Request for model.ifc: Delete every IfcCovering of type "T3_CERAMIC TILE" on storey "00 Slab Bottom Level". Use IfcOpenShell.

First a look at what the model holds.

```python
import ifcopenshell
import ifcopenshell.util.element

model = ifcopenshell.open("model.ifc")
print(model.schema)
storey = next(s for s in model.by_type("IfcBuildingStorey") if s.Name == "00 Slab Bottom Level")
coverings = [e for e in ifcopenshell.util.element.get_decomposition(storey) if e.is_a("IfcCovering")]
seen = {}
for e in coverings:
    element_type = ifcopenshell.util.element.get_type(e)
    name = element_type.Name if element_type not in (None, e) else None
    seen[name] = seen.get(name, 0) + 1
for name, count in sorted(seen.items(), key=str):
    print(count, "x", name)
```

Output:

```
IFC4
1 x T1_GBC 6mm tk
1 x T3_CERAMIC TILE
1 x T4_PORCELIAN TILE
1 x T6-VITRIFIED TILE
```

```python
import ifcopenshell
import ifcopenshell.api.root
import ifcopenshell.util.element

model = ifcopenshell.open("model.ifc")

storey = next(s for s in model.by_type("IfcBuildingStorey") if s.Name == "00 Slab Bottom Level")
coverings = [e for e in ifcopenshell.util.element.get_decomposition(storey) if e.is_a("IfcCovering")]
targets = [e for e in coverings if (t := ifcopenshell.util.element.get_type(e)) not in (None, e) and t.Name == "T3_CERAMIC TILE"]

for e in targets:
    ifcopenshell.api.root.remove_product(model, product=e)
print(len(targets), "removed")

model.write("model_rev.ifc")
```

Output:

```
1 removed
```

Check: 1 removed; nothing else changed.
